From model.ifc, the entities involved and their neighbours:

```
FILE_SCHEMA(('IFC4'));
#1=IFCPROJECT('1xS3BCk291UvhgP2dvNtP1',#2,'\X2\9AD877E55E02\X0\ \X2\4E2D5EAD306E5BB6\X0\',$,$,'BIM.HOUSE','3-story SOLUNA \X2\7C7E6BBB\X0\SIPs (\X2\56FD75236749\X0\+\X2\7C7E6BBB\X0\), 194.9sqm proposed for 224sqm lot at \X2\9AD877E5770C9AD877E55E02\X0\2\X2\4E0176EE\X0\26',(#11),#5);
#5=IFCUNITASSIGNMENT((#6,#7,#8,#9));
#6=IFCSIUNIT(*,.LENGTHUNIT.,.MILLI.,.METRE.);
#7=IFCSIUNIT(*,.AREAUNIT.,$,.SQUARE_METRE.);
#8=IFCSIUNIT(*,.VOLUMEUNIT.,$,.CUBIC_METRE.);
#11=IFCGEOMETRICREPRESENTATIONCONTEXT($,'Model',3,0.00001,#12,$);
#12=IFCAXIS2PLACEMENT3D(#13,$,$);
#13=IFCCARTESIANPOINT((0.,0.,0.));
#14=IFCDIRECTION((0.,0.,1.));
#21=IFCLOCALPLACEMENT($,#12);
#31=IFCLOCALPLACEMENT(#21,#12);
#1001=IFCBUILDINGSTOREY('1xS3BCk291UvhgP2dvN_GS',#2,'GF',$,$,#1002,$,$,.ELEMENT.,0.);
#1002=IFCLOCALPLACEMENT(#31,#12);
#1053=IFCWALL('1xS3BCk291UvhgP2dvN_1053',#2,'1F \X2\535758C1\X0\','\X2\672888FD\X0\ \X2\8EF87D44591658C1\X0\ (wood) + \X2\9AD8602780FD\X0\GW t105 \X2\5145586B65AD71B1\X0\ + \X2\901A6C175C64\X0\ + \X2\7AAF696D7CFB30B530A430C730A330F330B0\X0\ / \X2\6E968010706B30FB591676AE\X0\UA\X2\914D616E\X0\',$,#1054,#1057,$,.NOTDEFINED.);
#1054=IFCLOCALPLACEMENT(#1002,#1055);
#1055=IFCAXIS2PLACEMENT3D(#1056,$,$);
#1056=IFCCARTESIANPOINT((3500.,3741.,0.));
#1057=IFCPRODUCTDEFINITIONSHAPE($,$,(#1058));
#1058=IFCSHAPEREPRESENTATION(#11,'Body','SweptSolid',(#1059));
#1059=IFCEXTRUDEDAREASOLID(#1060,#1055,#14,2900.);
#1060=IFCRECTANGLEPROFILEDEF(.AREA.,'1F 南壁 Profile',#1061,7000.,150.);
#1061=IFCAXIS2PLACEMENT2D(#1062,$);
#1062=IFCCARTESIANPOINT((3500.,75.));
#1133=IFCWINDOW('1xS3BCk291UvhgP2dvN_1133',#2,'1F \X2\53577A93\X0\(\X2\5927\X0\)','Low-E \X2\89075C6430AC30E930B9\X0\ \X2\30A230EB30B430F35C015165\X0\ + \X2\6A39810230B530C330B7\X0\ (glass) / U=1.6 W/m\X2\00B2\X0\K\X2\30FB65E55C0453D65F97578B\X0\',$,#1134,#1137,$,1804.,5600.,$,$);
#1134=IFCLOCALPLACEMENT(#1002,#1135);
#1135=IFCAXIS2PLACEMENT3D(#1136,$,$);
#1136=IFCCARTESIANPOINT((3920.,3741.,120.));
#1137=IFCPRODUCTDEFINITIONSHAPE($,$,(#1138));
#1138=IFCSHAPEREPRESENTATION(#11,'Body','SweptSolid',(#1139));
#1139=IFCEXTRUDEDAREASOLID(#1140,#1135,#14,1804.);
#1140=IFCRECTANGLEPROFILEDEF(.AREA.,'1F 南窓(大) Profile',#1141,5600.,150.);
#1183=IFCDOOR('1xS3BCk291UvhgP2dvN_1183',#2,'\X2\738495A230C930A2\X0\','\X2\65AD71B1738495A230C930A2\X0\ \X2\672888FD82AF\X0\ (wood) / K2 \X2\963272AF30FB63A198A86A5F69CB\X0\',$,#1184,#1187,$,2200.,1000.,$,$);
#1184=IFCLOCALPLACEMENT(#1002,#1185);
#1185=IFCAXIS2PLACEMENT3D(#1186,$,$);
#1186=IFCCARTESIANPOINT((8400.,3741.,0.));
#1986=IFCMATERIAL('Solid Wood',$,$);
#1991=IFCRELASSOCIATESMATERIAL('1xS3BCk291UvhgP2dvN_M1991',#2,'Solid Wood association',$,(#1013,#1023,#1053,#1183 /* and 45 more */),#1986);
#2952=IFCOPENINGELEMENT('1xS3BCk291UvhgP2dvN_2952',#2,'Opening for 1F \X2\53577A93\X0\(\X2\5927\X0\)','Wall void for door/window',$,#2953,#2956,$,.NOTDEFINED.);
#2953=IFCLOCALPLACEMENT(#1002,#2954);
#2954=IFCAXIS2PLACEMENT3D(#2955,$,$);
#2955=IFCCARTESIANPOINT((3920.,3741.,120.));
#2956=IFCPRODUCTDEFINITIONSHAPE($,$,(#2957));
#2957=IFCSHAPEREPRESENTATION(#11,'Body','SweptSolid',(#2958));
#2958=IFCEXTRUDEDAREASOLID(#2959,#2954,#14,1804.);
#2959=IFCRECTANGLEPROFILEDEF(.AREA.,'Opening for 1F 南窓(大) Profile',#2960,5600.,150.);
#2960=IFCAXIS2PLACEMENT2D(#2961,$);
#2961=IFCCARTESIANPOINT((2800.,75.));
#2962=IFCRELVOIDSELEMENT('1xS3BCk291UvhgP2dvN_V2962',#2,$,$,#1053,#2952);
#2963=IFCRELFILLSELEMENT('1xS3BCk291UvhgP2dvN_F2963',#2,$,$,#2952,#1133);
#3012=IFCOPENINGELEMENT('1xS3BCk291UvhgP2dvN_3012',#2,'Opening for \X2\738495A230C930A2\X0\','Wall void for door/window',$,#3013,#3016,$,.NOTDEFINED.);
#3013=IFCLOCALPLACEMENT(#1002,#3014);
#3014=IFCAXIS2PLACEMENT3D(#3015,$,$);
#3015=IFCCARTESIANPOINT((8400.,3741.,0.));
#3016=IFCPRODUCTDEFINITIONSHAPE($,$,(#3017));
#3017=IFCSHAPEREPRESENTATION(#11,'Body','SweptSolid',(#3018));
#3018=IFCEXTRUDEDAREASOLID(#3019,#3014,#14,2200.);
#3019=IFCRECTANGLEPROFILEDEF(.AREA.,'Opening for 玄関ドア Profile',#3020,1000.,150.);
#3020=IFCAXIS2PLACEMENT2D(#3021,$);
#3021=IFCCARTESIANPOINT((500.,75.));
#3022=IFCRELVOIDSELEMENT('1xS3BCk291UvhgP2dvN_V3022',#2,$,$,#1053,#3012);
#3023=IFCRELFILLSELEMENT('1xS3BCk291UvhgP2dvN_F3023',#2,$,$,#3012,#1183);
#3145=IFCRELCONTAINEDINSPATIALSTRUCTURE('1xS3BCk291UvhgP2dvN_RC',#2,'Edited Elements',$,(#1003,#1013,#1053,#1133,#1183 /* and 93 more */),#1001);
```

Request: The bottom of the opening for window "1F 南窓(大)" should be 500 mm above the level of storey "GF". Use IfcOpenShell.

```python
import numpy as np
import ifcopenshell
import ifcopenshell.api.geometry
import ifcopenshell.geom
import ifcopenshell.util.element
import ifcopenshell.util.placement
import ifcopenshell.util.shape
import ifcopenshell.util.unit

model = ifcopenshell.open("model.ifc")
unit_scale = ifcopenshell.util.unit.calculate_unit_scale(model)

window = model.by_guid("1xS3BCk291UvhgP2dvN_1133")
opening = window.FillsVoids[0].RelatingOpeningElement
storey = ifcopenshell.util.element.get_container(window, ifc_class="IfcBuildingStorey")
level = ifcopenshell.util.placement.get_local_placement(storey.ObjectPlacement)[2, 3]

# The opening's origin need not be at the sill, so measure its lowest point.
shape = ifcopenshell.geom.create_shape(ifcopenshell.geom.settings(), opening)
bottom = ifcopenshell.util.shape.get_shape_bottom_elevation(shape, shape.geometry) / unit_scale
dz = level + 0.5 / unit_scale - bottom

shift = np.array([0.0, 0.0, dz])
# The window is not placed relative to its opening, so move both.
for product in (opening, window):
    matrix = ifcopenshell.util.placement.get_local_placement(product.ObjectPlacement)
    matrix[:3, 3] += shift
    ifcopenshell.api.geometry.edit_object_placement(model, product=product, matrix=matrix, is_si=False)

print(f"moved by {dz * unit_scale:+.3f} m")

model.write("model-out.ifc")
```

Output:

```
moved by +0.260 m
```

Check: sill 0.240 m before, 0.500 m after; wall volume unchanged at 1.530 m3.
